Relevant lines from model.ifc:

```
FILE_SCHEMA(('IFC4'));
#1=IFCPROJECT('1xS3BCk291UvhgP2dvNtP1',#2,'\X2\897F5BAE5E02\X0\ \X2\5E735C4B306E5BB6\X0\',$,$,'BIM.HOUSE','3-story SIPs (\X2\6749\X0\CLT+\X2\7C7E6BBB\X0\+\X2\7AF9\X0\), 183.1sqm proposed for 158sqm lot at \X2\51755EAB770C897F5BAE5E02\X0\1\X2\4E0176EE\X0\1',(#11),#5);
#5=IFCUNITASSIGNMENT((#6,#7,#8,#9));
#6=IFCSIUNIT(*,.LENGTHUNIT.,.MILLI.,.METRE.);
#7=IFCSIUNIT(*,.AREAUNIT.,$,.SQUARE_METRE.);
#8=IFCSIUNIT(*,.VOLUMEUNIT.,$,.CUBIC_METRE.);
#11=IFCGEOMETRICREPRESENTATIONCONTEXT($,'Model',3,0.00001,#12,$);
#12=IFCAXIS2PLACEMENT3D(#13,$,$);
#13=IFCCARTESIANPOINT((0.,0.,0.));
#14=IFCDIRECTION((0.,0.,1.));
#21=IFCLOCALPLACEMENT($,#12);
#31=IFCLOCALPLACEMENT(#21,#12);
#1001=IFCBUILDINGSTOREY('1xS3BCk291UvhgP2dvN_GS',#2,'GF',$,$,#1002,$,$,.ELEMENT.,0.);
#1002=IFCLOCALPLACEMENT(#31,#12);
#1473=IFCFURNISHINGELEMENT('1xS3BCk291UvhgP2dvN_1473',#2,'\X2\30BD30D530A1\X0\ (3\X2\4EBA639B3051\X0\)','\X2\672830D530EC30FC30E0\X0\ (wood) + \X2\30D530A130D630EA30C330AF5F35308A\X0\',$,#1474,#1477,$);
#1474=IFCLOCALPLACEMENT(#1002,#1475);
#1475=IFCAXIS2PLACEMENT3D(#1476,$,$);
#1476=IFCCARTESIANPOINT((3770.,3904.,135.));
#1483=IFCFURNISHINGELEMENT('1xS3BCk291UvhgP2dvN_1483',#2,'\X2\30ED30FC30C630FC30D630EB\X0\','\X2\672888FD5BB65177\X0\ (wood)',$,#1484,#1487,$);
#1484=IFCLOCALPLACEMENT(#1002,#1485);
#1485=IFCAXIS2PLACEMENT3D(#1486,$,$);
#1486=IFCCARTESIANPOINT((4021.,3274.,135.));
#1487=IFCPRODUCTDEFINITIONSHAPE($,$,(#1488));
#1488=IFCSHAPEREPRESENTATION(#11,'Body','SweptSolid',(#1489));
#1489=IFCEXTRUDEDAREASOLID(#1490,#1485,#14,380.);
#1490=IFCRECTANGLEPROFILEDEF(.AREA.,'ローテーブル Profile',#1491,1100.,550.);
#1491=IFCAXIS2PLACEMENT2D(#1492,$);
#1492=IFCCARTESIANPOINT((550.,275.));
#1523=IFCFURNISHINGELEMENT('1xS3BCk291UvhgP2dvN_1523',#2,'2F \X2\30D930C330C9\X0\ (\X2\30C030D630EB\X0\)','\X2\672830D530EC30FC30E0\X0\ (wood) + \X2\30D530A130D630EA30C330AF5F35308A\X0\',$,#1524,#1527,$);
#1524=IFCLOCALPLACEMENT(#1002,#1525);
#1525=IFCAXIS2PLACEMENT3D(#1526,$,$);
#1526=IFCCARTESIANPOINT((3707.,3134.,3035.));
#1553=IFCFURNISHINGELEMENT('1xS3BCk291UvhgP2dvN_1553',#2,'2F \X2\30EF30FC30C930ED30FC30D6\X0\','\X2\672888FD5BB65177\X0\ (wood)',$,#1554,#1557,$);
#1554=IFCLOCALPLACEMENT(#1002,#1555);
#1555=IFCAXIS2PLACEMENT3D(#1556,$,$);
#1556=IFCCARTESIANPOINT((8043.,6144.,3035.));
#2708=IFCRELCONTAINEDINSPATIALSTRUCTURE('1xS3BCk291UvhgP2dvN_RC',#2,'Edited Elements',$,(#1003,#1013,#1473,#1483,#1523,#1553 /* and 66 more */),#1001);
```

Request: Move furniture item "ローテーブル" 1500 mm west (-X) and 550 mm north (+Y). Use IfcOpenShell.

```python
import ifcopenshell
import ifcopenshell.api.geometry
import ifcopenshell.util.placement
import ifcopenshell.util.unit

model = ifcopenshell.open("model.ifc")
unit_scale = ifcopenshell.util.unit.calculate_unit_scale(model)

item = model.by_guid("1xS3BCk291UvhgP2dvN_1483")
matrix = ifcopenshell.util.placement.get_local_placement(item.ObjectPlacement)
matrix[0, 3] -= 1.5 / unit_scale
matrix[1, 3] += 0.55 / unit_scale
ifcopenshell.api.geometry.edit_object_placement(model, product=item, matrix=matrix, is_si=False)

print(ifcopenshell.util.placement.get_local_placement(item.ObjectPlacement).round(3) + 0.0)

model.write("model_edited.ifc")
```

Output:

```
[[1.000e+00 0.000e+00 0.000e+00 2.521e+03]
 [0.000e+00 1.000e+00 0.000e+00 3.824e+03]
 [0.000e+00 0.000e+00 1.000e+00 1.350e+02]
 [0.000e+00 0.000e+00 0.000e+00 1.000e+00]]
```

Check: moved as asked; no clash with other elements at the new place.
